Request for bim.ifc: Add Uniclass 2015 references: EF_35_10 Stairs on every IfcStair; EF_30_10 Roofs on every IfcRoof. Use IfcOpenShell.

First a look at what the model holds.

```python
import ifcopenshell

model = ifcopenshell.open("bim.ifc")
print(model.schema)
print("classifications:", [c.Name for c in model.by_type("IfcClassification")])
for ifc_class in ("IfcDoor", "IfcRoof", "IfcStair", "IfcWall", "IfcWindow"):
    print(ifc_class, len(model.by_type(ifc_class)))
```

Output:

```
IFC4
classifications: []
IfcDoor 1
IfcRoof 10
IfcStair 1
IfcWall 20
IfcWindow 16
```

```python
import ifcopenshell
import ifcopenshell.api.classification

model = ifcopenshell.open("bim.ifc")

system = ifcopenshell.api.classification.add_classification(model, classification="Uniclass 2015")

codes = {
    "IfcStair": ("EF_35_10", "Stairs"),
    "IfcRoof": ("EF_30_10", "Roofs"),
}
for ifc_class, (code, name) in codes.items():
    products = model.by_type(ifc_class)
    ifcopenshell.api.classification.add_reference(
        model, products=products, classification=system, identification=code, name=name
    )
    print(code, len(products))

model.write("bim_edited.ifc")
```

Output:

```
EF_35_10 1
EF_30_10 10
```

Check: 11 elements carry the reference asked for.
